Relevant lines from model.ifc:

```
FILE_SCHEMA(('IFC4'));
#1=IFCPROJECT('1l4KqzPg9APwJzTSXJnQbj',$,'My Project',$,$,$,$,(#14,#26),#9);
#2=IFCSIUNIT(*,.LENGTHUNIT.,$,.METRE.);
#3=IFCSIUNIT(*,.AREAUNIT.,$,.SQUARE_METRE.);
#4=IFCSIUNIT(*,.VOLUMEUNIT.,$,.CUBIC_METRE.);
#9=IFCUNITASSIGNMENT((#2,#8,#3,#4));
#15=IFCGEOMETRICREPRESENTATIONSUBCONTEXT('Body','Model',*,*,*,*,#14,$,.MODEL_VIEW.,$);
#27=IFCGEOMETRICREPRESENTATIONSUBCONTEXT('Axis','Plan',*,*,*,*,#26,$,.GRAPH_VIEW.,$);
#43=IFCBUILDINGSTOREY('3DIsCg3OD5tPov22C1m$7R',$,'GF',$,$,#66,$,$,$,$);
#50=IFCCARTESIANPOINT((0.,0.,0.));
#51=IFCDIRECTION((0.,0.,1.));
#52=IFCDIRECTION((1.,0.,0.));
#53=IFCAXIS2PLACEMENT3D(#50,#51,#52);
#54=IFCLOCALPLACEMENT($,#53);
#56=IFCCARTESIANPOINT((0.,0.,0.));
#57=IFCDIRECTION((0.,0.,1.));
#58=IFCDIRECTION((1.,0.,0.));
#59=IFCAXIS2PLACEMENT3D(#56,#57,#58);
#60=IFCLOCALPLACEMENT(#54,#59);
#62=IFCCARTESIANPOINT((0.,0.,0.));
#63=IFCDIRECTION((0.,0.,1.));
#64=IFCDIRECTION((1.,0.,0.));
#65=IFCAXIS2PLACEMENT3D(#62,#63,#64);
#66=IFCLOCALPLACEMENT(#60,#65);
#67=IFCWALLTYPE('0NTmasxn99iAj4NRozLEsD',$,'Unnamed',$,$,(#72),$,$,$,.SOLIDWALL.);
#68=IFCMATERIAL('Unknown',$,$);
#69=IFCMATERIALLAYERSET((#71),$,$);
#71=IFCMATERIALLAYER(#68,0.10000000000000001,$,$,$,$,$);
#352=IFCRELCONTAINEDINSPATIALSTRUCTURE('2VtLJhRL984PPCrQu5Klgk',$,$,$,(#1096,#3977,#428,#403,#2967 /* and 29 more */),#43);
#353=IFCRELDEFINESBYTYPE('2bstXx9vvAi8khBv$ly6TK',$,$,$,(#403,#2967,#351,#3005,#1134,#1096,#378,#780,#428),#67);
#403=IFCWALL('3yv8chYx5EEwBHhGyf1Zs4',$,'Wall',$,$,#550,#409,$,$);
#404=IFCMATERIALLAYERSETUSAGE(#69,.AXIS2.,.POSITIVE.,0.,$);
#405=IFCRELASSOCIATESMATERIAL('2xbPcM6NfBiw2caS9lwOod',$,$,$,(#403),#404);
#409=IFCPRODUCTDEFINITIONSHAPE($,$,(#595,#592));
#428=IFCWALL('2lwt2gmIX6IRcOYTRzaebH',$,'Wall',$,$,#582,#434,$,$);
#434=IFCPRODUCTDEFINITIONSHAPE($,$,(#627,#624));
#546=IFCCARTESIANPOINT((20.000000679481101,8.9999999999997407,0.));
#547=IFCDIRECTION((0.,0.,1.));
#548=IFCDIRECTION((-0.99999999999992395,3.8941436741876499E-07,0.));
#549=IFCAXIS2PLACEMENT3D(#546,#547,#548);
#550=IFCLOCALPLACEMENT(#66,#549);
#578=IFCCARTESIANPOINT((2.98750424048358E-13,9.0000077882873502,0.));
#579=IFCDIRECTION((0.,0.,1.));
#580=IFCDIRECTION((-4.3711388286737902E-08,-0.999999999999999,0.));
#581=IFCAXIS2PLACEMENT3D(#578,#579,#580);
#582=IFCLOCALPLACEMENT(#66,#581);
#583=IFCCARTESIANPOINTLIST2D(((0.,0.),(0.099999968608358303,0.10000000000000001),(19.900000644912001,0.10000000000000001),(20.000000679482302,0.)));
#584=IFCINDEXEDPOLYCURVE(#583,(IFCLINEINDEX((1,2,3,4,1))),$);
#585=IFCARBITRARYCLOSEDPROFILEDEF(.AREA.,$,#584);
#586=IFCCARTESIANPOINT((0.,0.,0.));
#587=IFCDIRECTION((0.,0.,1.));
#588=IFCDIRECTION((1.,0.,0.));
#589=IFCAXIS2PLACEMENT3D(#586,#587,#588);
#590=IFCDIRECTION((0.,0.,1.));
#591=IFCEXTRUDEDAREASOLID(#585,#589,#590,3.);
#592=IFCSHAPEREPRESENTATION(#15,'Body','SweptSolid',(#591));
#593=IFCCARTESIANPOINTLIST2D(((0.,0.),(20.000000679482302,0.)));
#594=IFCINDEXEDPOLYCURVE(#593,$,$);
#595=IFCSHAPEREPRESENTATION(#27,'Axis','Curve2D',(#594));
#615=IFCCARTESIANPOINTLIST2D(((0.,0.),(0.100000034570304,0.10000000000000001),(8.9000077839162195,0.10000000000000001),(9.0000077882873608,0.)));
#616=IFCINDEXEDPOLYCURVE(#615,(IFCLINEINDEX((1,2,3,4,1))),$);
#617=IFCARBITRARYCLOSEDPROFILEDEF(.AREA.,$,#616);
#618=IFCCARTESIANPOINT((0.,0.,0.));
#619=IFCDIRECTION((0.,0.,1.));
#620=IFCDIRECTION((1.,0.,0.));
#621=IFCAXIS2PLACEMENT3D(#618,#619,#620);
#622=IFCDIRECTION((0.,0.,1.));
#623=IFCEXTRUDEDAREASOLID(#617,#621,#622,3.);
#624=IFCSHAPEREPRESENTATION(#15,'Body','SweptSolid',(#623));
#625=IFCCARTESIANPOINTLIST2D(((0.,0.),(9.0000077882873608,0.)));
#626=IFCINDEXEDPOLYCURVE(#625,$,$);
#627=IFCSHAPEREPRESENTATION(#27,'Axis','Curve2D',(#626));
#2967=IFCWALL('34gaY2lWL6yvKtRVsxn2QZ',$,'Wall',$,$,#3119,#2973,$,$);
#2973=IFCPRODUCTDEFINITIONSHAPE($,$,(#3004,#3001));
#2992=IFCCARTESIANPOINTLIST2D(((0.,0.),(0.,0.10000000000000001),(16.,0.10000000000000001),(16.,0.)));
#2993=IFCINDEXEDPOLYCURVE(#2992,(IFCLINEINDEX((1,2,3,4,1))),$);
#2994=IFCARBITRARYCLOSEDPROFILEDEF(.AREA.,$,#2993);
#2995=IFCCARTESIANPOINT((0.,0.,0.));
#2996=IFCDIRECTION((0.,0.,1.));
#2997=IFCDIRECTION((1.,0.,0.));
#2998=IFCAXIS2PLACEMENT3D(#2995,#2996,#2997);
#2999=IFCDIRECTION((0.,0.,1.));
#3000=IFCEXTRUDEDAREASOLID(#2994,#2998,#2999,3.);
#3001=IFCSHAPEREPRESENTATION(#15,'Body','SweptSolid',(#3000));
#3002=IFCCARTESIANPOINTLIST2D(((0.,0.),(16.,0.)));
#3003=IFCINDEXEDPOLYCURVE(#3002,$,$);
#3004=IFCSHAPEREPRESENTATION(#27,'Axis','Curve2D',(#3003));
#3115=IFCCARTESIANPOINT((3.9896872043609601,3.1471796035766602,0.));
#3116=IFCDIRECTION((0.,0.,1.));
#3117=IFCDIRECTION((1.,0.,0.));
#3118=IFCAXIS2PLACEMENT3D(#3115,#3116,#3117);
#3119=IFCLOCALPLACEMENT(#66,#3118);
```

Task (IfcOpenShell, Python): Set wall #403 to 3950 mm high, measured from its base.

```python
import ifcopenshell
import ifcopenshell.geom
import ifcopenshell.util.representation
import ifcopenshell.util.shape

model = ifcopenshell.open("model.ifc")
settings = ifcopenshell.geom.settings()


def volume(element):
    """Net volume in cubic metres, openings subtracted."""
    shape = ifcopenshell.geom.create_shape(settings, element)
    return ifcopenshell.util.shape.get_volume(shape.geometry)


wall = model.by_guid("3yv8chYx5EEwBHhGyf1Zs4")
before = volume(wall)

body = ifcopenshell.util.representation.get_representation(wall, "Model", "Body")
solid = body.Items[0]
old_height = solid.Depth
solid.Depth = 3.95
after = volume(wall)

print(f"height {old_height:g} -> {solid.Depth:g}, volume {before:.3f} -> {after:.3f} m3")

model.write("model_rev.ifc")
```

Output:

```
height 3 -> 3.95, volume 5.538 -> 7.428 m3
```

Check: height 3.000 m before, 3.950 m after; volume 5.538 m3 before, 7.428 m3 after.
